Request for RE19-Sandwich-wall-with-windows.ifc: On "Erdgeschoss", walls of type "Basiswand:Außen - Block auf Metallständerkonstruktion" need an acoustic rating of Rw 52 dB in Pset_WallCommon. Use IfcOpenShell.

First a look at what the model holds.

```python
import ifcopenshell
import ifcopenshell.util.element

model = ifcopenshell.open("RE19-Sandwich-wall-with-windows.ifc")
print(model.schema)
storey = next(s for s in model.by_type("IfcBuildingStorey") if s.Name == "Erdgeschoss")
walls = [e for e in ifcopenshell.util.element.get_decomposition(storey) if e.is_a("IfcWall")]
seen = {}
for e in walls:
    element_type = ifcopenshell.util.element.get_type(e)
    key = (element_type.Name if element_type != e and element_type else None, ifcopenshell.util.element.get_pset(e, "Pset_WallCommon", "AcousticRating"))
    seen[key] = seen.get(key, 0) + 1
for (name, value), count in sorted(seen.items(), key=str):
    print(count, "x", name, "|", value)
```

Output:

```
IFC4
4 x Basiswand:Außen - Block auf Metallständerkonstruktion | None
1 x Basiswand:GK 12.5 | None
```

```python
import ifcopenshell
import ifcopenshell.api.pset
import ifcopenshell.util.element

model = ifcopenshell.open("RE19-Sandwich-wall-with-windows.ifc")

storey = next(s for s in model.by_type("IfcBuildingStorey") if s.Name == "Erdgeschoss")
walls = [e for e in ifcopenshell.util.element.get_decomposition(storey) if e.is_a("IfcWall")]

count = 0
for e in walls:
    element_type = ifcopenshell.util.element.get_type(e)
    if element_type in (None, e) or element_type.Name != "Basiswand:Außen - Block auf Metallständerkonstruktion":
        continue
    # add_pset returns the element's existing set when there is one.
    pset = ifcopenshell.api.pset.add_pset(model, product=e, name="Pset_WallCommon")
    ifcopenshell.api.pset.edit_pset(model, pset=pset, properties={"AcousticRating": "Rw 52 dB"})
    count += 1

print(count, "walls updated")

model.write("RE19-Sandwich-wall-with-windows_rev.ifc")
```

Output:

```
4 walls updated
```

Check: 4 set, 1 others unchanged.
